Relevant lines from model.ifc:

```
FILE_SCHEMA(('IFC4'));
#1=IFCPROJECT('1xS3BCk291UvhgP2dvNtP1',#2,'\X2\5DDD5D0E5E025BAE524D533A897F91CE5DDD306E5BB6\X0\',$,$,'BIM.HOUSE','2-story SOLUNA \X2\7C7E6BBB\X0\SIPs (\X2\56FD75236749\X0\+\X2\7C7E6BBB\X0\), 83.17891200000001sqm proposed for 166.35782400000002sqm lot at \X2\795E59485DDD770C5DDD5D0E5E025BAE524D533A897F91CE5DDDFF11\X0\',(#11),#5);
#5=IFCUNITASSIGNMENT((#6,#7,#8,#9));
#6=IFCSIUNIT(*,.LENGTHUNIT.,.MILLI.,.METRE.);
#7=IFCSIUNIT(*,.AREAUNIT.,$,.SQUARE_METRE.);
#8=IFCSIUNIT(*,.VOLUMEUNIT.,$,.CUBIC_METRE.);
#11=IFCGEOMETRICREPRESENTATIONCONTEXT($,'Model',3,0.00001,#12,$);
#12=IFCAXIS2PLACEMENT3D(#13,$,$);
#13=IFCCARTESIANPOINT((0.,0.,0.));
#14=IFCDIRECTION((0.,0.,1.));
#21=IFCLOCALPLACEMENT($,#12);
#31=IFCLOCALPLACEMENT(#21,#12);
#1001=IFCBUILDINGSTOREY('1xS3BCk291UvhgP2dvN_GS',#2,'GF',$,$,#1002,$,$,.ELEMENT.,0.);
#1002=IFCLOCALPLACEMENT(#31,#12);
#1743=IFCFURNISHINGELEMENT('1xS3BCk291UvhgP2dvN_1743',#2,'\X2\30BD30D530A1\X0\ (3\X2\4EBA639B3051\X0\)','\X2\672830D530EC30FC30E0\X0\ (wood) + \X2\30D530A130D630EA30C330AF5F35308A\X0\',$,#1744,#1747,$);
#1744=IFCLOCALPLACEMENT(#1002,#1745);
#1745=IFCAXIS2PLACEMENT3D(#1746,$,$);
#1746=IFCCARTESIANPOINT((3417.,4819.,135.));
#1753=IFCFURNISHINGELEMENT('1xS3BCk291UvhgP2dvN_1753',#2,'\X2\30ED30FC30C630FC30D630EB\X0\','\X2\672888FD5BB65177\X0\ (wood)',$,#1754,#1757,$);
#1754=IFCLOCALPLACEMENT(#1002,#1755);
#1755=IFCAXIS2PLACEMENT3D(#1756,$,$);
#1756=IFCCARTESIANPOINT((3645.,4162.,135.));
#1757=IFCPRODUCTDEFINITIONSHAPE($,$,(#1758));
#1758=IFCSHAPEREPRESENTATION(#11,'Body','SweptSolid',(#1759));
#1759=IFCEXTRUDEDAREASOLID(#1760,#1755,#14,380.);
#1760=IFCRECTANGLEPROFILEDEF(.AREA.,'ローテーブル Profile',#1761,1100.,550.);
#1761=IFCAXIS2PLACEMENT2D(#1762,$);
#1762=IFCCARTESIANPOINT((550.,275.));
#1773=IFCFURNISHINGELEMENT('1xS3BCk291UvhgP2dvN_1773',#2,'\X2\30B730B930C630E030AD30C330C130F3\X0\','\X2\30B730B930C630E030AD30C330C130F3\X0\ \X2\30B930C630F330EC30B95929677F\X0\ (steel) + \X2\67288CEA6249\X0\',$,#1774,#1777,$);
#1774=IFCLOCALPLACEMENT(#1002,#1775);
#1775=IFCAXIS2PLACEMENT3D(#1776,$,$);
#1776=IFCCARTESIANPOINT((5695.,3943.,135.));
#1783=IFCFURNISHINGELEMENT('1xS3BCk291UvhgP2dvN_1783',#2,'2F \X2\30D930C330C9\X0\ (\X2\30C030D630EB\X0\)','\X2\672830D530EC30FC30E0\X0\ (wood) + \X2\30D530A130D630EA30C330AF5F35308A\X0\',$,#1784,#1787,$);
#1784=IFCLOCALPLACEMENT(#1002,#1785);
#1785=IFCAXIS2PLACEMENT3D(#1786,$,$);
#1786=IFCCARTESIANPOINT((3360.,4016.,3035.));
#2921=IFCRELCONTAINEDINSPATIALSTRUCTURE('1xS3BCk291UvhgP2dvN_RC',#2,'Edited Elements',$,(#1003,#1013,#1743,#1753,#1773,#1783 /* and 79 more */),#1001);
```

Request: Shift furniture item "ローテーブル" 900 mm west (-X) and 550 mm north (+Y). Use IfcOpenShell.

```python
import ifcopenshell
import ifcopenshell.api.geometry
import ifcopenshell.util.placement

model = ifcopenshell.open("model.ifc")

item = model.by_id(1753)
matrix = ifcopenshell.util.placement.get_local_placement(item.ObjectPlacement)
matrix[0, 3] -= 900.0
matrix[1, 3] += 550.0
ifcopenshell.api.geometry.edit_object_placement(model, product=item, matrix=matrix, is_si=False)

print(ifcopenshell.util.placement.get_local_placement(item.ObjectPlacement).round(3) + 0.0)

model.write("model_rev.ifc")
```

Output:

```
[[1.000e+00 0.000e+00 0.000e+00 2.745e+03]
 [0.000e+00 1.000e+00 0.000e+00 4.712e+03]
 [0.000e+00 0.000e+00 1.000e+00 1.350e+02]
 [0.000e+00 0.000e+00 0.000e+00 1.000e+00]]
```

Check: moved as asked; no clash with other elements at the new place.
